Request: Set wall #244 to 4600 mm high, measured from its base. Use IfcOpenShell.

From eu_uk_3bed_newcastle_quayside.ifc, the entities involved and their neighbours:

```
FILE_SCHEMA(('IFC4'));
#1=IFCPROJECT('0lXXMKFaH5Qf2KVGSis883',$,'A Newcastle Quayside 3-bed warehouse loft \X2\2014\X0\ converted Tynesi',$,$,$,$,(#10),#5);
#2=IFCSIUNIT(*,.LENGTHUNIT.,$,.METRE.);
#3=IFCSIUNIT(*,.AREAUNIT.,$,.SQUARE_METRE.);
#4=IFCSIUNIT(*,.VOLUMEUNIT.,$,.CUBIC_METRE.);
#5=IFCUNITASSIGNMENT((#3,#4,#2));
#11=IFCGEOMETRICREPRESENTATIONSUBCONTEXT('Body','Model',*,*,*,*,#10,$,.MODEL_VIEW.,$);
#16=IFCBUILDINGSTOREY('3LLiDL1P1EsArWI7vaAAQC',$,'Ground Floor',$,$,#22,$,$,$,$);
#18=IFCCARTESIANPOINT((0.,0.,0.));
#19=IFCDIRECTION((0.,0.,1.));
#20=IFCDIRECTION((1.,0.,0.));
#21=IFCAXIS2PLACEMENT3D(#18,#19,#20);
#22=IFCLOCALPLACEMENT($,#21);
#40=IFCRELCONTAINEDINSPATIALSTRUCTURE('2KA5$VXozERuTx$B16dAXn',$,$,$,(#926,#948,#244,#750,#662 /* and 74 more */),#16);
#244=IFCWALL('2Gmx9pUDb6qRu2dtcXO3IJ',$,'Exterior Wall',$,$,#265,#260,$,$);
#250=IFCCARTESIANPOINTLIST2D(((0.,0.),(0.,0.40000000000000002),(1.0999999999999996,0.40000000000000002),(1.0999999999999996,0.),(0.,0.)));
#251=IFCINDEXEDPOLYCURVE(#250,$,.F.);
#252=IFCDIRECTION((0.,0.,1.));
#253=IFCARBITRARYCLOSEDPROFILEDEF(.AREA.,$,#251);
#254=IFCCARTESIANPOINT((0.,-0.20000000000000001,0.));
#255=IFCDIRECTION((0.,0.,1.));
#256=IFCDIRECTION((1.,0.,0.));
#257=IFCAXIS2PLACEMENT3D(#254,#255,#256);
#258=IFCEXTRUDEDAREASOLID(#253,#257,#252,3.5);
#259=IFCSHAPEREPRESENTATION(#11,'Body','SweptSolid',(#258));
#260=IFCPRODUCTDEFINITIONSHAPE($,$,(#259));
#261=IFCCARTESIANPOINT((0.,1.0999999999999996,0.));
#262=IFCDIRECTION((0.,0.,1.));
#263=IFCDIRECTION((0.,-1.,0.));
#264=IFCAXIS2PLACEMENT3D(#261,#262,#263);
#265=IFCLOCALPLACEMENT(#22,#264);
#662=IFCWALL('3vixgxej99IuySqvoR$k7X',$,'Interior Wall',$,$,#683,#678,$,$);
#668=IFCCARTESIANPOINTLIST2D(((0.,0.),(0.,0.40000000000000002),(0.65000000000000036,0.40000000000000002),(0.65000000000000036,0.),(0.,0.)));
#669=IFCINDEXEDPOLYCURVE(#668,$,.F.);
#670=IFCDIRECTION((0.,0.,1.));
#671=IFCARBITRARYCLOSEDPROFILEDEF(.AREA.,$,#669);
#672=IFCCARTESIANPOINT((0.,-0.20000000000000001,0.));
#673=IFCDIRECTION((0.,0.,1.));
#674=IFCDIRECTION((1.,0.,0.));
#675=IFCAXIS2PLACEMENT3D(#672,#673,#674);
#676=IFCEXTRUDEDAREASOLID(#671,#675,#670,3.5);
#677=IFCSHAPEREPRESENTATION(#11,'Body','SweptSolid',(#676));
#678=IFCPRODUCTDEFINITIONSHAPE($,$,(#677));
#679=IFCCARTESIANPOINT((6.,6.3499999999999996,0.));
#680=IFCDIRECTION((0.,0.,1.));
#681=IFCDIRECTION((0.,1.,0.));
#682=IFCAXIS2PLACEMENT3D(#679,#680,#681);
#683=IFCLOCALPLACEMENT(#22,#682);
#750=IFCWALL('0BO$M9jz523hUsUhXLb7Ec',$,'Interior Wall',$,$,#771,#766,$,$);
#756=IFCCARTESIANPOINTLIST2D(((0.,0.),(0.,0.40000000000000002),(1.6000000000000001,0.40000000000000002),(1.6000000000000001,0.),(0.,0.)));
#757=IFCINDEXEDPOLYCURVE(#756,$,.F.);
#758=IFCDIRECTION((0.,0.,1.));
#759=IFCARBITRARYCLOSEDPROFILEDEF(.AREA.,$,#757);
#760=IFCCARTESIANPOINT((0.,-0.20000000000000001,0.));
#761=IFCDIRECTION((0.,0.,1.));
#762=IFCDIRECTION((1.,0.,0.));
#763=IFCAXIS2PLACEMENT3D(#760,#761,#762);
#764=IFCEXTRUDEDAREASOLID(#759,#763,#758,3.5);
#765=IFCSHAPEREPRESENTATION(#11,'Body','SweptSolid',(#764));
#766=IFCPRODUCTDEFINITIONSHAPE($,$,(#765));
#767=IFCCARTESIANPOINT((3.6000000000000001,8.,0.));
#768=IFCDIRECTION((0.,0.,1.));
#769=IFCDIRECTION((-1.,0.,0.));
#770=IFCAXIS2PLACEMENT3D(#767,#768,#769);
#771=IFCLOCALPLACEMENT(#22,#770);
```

```python
import ifcopenshell
import ifcopenshell.geom
import ifcopenshell.util.representation
import ifcopenshell.util.shape

model = ifcopenshell.open("eu_uk_3bed_newcastle_quayside.ifc")
settings = ifcopenshell.geom.settings()


def volume(element):
    """Net volume in cubic metres, openings subtracted."""
    shape = ifcopenshell.geom.create_shape(settings, element)
    return ifcopenshell.util.shape.get_volume(shape.geometry)


wall = model.by_guid("2Gmx9pUDb6qRu2dtcXO3IJ")
before = volume(wall)

body = ifcopenshell.util.representation.get_representation(wall, "Model", "Body")
solid = body.Items[0]
old_height = solid.Depth
solid.Depth = 4.6
after = volume(wall)

print(f"height {old_height:g} -> {solid.Depth:g}, volume {before:.3f} -> {after:.3f} m3")

model.write("eu_uk_3bed_newcastle_quayside_updated.ifc")
```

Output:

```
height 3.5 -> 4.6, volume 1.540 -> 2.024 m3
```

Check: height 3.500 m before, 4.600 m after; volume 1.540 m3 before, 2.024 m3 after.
